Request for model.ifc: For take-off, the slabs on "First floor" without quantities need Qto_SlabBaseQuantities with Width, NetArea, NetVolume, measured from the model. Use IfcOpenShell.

First a look at what the model holds.

```python
import ifcopenshell
import ifcopenshell.util.element
import ifcopenshell.util.unit

model = ifcopenshell.open("model.ifc")
print(model.schema)
for unit_type in ("LENGTHUNIT", "AREAUNIT", "VOLUMEUNIT"):
    print(unit_type, ifcopenshell.util.unit.calculate_unit_scale(model, unit_type))
storey = next(s for s in model.by_type("IfcBuildingStorey") if s.Name == "First floor")
slabs = [e for e in ifcopenshell.util.element.get_decomposition(storey) if e.is_a("IfcSlab")]
for e in sorted(slabs, key=lambda e: e.id()):
    print(e.id(), e.is_a(), e.Name, list(ifcopenshell.util.element.get_psets(e, qtos_only=True)), sep=" | ")
```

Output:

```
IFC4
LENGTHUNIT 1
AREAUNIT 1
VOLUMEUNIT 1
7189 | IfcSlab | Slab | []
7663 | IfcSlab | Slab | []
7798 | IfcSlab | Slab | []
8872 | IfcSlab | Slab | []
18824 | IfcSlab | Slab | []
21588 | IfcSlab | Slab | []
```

```python
import ifcopenshell
import ifcopenshell.api.pset
import ifcopenshell.geom
import ifcopenshell.util.element
import ifcopenshell.util.shape
import ifcopenshell.util.unit

model = ifcopenshell.open("model.ifc")
unit_scale = ifcopenshell.util.unit.calculate_unit_scale(model)
area_scale = ifcopenshell.util.unit.calculate_unit_scale(model, "AREAUNIT")
volume_scale = ifcopenshell.util.unit.calculate_unit_scale(model, "VOLUMEUNIT")
settings = ifcopenshell.geom.settings()

storey = next(s for s in model.by_type("IfcBuildingStorey") if s.Name == "First floor")
slabs = [e for e in ifcopenshell.util.element.get_decomposition(storey) if e.is_a("IfcSlab")]

for e in sorted(slabs, key=lambda e: e.id()):
    if ifcopenshell.util.element.get_psets(e, qtos_only=True, should_inherit=False):
        continue
    # Geometry comes back in metres, in the element's own axes.
    shape = ifcopenshell.geom.create_shape(settings, e)
    values = {
        "Width": ifcopenshell.util.shape.get_z(shape.geometry) / unit_scale,
        "NetArea": ifcopenshell.util.shape.get_footprint_area(shape.geometry) / area_scale,
        "NetVolume": ifcopenshell.util.shape.get_volume(shape.geometry) / volume_scale,
    }
    qto = ifcopenshell.api.pset.add_qto(model, product=e, name="Qto_SlabBaseQuantities")
    ifcopenshell.api.pset.edit_qto(model, qto=qto, properties=values)
    print(e.id(), {k: round(v, 3) for k, v in values.items()})

model.write("model-out.ifc")
```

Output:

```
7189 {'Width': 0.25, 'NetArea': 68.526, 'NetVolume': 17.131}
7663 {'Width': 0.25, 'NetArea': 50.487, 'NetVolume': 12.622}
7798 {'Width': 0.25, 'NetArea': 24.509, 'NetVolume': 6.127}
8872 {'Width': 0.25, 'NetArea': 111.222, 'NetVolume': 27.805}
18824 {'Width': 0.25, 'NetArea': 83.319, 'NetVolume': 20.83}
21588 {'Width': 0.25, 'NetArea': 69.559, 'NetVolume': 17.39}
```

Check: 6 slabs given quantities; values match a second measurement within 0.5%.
